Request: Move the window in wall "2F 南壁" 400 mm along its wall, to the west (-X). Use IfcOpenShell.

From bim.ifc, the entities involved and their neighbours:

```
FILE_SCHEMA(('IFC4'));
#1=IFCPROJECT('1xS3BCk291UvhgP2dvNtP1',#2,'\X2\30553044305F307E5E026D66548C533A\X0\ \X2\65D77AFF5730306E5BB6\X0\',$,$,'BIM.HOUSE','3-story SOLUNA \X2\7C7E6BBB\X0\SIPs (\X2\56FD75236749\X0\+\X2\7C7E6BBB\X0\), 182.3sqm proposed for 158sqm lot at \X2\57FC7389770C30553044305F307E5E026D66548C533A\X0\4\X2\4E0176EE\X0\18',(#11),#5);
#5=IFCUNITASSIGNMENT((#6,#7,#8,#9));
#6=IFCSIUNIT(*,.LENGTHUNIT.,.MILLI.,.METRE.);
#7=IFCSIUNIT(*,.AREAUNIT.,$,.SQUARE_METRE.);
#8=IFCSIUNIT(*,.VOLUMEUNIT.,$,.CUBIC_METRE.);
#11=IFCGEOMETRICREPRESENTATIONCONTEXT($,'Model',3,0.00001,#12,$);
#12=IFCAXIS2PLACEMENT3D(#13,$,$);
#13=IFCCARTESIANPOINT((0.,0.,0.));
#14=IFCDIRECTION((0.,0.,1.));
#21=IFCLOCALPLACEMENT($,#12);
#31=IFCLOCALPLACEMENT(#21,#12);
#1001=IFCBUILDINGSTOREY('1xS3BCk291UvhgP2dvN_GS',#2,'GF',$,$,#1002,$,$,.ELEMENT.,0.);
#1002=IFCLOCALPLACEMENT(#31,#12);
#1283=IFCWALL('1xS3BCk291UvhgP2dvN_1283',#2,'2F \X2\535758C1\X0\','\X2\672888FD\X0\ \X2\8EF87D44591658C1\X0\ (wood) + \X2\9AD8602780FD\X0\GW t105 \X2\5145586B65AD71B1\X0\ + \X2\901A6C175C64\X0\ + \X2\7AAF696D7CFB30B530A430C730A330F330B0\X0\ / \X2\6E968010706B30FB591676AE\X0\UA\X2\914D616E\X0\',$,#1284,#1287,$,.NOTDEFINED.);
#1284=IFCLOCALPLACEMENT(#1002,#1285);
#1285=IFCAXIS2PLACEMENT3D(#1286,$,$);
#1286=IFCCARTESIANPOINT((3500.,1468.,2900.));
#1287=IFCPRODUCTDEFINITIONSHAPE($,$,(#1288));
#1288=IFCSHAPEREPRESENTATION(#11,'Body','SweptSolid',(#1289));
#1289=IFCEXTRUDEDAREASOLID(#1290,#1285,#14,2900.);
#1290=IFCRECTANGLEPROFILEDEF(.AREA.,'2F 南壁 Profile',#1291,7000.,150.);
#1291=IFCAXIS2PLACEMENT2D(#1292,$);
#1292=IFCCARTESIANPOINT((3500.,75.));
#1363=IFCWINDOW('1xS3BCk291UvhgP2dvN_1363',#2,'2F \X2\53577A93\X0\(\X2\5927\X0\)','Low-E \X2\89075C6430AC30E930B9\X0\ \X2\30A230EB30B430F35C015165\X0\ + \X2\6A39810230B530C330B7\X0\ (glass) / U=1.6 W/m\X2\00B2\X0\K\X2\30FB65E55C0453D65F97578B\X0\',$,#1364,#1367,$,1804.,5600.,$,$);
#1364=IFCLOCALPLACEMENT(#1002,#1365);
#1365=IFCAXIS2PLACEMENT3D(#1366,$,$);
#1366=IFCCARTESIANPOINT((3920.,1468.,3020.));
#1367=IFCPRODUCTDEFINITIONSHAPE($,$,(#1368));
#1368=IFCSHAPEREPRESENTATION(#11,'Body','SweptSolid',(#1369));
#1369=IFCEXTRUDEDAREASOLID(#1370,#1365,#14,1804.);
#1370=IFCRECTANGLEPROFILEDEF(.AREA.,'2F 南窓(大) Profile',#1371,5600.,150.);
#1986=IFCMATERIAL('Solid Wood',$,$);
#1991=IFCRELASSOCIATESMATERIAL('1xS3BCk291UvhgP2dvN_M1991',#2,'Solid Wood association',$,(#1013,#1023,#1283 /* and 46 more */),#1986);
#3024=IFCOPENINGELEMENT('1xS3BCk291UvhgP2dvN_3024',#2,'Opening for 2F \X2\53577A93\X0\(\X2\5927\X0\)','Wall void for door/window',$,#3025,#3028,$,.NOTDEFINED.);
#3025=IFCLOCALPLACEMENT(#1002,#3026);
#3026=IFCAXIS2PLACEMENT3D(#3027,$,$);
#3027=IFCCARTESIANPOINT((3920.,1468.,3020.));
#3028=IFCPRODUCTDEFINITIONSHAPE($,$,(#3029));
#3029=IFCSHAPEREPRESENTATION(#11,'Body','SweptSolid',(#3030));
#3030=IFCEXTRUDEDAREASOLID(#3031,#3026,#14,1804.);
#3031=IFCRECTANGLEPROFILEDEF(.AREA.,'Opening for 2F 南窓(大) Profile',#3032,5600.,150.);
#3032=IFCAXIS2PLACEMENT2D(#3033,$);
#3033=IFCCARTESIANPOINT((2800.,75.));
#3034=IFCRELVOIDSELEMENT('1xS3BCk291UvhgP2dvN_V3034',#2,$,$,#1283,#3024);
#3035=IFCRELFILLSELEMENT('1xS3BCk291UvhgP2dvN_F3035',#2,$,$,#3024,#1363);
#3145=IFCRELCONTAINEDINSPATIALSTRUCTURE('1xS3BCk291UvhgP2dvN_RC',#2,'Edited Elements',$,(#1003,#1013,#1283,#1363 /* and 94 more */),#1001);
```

```python
import ifcopenshell
import ifcopenshell.api.geometry
import ifcopenshell.util.placement
import ifcopenshell.util.unit

model = ifcopenshell.open("bim.ifc")
unit_scale = ifcopenshell.util.unit.calculate_unit_scale(model)

window = model.by_id(1363)
opening = window.FillsVoids[0].RelatingOpeningElement
wall = opening.VoidsElements[0].RelatingBuildingElement

wall_matrix = ifcopenshell.util.placement.get_local_placement(wall.ObjectPlacement)
shift = wall_matrix[:3, 0] * -0.4 / unit_scale
before = ifcopenshell.util.placement.get_local_placement(window.ObjectPlacement)[:3, 3].copy()

# The window is not placed relative to its opening, so move both.
for product in (opening, window):
    matrix = ifcopenshell.util.placement.get_local_placement(product.ObjectPlacement)
    matrix[:3, 3] += shift
    ifcopenshell.api.geometry.edit_object_placement(model, product=product, matrix=matrix, is_si=False)

after = ifcopenshell.util.placement.get_local_placement(window.ObjectPlacement)[:3, 3]
print("window moved by", (after - before).round(3) + 0.0)

model.write("bim_edited.ifc")
```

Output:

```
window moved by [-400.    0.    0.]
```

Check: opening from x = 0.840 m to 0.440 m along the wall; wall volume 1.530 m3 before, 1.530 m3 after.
